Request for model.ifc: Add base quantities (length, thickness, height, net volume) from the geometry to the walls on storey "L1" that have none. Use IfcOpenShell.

First a look at what the model holds.

```python
import ifcopenshell
import ifcopenshell.util.element
import ifcopenshell.util.unit

model = ifcopenshell.open("model.ifc")
print(model.schema)
for unit_type in ("LENGTHUNIT", "AREAUNIT", "VOLUMEUNIT"):
    print(unit_type, ifcopenshell.util.unit.calculate_unit_scale(model, unit_type))
storey = next(s for s in model.by_type("IfcBuildingStorey") if s.Name == "L1")
walls = [e for e in ifcopenshell.util.element.get_decomposition(storey) if e.is_a("IfcWall")]
for e in sorted(walls, key=lambda e: e.id()):
    print(e.id(), e.is_a(), e.Name, list(ifcopenshell.util.element.get_psets(e, qtos_only=True)), sep=" | ")
```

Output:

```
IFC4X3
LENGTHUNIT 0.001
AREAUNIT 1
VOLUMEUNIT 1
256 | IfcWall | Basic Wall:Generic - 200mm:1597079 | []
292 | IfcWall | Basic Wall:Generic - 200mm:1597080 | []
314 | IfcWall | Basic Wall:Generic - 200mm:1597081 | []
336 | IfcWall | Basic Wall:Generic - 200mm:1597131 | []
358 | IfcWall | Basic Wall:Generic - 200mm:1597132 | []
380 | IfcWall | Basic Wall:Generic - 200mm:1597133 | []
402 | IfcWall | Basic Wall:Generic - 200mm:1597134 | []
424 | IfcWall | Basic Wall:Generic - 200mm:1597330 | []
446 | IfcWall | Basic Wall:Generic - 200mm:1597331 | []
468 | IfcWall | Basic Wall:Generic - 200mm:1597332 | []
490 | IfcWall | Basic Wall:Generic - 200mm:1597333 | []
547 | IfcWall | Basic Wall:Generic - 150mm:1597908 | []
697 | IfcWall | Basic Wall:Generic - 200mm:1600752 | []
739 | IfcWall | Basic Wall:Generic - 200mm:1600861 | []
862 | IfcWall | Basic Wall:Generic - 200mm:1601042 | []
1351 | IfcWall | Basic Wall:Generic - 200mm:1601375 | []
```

```python
import ifcopenshell
import ifcopenshell.api.pset
import ifcopenshell.geom
import ifcopenshell.util.element
import ifcopenshell.util.shape
import ifcopenshell.util.unit

model = ifcopenshell.open("model.ifc")
unit_scale = ifcopenshell.util.unit.calculate_unit_scale(model)
volume_scale = ifcopenshell.util.unit.calculate_unit_scale(model, "VOLUMEUNIT")
settings = ifcopenshell.geom.settings()

storey = next(s for s in model.by_type("IfcBuildingStorey") if s.Name == "L1")
walls = [e for e in ifcopenshell.util.element.get_decomposition(storey) if e.is_a("IfcWall")]

for e in sorted(walls, key=lambda e: e.id()):
    if ifcopenshell.util.element.get_psets(e, qtos_only=True, should_inherit=False):
        continue
    # Geometry comes back in metres, in the element's own axes.
    shape = ifcopenshell.geom.create_shape(settings, e)
    values = {
        "Length": ifcopenshell.util.shape.get_x(shape.geometry) / unit_scale,
        "Width": ifcopenshell.util.shape.get_y(shape.geometry) / unit_scale,
        "Height": ifcopenshell.util.shape.get_z(shape.geometry) / unit_scale,
        "NetVolume": ifcopenshell.util.shape.get_volume(shape.geometry) / volume_scale,
    }
    qto = ifcopenshell.api.pset.add_qto(model, product=e, name="Qto_WallBaseQuantities")
    ifcopenshell.api.pset.edit_qto(model, qto=qto, properties=values)
    print(e.id(), {k: round(v, 3) for k, v in values.items()})

model.write("model-out.ifc")
```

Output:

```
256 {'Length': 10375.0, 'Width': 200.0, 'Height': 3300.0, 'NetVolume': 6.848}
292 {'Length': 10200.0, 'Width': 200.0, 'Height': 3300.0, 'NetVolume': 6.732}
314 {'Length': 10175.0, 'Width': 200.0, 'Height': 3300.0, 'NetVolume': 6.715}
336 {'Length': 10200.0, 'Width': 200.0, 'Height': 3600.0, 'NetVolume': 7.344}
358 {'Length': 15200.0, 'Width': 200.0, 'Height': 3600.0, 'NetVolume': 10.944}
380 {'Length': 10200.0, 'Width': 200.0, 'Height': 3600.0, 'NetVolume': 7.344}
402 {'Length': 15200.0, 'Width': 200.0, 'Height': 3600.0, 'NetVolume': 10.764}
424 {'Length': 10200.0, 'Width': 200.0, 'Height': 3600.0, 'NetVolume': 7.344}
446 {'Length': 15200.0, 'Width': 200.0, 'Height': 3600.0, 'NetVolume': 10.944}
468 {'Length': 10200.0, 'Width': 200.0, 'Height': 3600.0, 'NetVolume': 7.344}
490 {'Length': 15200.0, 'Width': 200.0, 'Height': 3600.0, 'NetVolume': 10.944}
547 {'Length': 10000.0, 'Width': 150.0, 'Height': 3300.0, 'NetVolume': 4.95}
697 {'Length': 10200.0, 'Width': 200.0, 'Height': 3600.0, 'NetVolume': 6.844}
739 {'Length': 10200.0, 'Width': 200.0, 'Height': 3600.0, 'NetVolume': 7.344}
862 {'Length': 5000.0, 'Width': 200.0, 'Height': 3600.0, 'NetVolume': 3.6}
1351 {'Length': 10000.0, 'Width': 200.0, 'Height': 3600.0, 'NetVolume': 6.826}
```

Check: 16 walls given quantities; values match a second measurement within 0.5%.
